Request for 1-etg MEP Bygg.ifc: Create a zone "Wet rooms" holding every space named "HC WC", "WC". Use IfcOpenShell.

First a look at what the model holds.

```python
import ifcopenshell

model = ifcopenshell.open("1-etg MEP Bygg.ifc")
print(model.schema)
seen = {}
for space in model.by_type("IfcSpace"):
    seen[space.LongName] = seen.get(space.LongName, 0) + 1
for name, count in sorted(seen.items(), key=str):
    print(count, "x", name)
print("zones:", [z.Name for z in model.by_type("IfcZone")][:20])
```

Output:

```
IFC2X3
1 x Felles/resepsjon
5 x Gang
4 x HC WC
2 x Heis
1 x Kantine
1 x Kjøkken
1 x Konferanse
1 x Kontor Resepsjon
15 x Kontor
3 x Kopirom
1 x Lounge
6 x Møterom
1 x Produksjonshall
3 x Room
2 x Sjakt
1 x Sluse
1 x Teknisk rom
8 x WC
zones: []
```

```python
import ifcopenshell
import ifcopenshell.api.group
import ifcopenshell.api.root

model = ifcopenshell.open("1-etg MEP Bygg.ifc")

names = {"HC WC", "WC"}
spaces = [s for s in model.by_type("IfcSpace") if s.LongName in names]

zone = ifcopenshell.api.root.create_entity(model, ifc_class="IfcZone", name="Wet rooms")
ifcopenshell.api.group.assign_group(model, products=spaces, group=zone)
print(len(spaces), "spaces in", zone.Name)

model.write("1-etg MEP Bygg_updated.ifc")
```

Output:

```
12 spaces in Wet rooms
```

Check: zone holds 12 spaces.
